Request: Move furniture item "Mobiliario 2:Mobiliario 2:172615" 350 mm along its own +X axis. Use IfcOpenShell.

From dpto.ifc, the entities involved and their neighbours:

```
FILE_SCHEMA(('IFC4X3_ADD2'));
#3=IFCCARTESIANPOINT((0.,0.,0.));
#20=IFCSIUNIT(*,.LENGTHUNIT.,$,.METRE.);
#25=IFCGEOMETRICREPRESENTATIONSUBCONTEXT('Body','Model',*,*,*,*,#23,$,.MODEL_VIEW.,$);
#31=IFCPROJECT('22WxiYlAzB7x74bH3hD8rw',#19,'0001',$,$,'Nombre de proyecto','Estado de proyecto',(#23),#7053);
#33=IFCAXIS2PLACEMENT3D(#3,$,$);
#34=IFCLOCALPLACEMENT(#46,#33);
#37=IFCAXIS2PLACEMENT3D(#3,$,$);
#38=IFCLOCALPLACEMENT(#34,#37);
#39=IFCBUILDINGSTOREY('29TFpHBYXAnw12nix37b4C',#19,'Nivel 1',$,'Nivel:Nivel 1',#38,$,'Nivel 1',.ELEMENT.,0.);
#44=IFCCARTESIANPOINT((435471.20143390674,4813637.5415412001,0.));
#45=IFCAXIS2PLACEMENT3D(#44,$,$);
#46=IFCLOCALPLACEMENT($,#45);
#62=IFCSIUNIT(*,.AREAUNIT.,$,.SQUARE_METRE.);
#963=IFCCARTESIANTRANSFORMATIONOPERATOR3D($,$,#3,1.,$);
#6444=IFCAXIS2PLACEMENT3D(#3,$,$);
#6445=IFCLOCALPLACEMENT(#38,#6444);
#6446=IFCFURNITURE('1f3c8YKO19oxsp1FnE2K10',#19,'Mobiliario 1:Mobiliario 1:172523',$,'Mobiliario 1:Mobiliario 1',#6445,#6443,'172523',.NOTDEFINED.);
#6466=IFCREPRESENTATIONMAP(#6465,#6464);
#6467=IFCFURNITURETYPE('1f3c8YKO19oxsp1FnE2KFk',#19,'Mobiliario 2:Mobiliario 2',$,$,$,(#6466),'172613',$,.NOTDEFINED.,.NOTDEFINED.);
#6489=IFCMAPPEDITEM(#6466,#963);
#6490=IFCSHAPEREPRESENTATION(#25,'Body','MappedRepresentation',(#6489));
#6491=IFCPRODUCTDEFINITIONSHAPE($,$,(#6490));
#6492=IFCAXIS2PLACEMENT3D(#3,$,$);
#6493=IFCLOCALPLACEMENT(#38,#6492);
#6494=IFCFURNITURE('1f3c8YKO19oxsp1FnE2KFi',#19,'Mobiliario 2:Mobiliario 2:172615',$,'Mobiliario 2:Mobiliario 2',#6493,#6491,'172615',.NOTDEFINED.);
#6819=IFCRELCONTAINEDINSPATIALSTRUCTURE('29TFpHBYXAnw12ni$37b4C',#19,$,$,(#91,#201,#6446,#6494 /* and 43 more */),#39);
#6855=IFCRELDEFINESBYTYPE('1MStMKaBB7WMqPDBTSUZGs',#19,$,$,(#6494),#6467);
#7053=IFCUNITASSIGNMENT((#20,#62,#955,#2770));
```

```python
import ifcopenshell
import ifcopenshell.api.geometry
import ifcopenshell.util.placement
import ifcopenshell.util.unit

model = ifcopenshell.open("dpto.ifc")
unit_scale = ifcopenshell.util.unit.calculate_unit_scale(model)

item = model.by_guid("1f3c8YKO19oxsp1FnE2KFi")
matrix = ifcopenshell.util.placement.get_local_placement(item.ObjectPlacement)
matrix[:3, 3] += matrix[:3, 0] * 0.35 / unit_scale
ifcopenshell.api.geometry.edit_object_placement(model, product=item, matrix=matrix, is_si=False)

print(ifcopenshell.util.placement.get_local_placement(item.ObjectPlacement).round(3) + 0.0)

model.write("dpto_v2.ifc")
```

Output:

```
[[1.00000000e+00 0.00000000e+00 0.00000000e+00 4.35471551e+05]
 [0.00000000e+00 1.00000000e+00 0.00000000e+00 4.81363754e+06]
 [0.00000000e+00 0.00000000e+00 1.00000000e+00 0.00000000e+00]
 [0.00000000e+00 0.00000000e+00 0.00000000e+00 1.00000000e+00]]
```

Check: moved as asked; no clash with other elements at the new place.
